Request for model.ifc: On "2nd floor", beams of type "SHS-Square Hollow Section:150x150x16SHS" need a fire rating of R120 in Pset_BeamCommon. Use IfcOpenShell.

First a look at what the model holds.

```python
import ifcopenshell
import ifcopenshell.util.element

model = ifcopenshell.open("model.ifc")
print(model.schema)
storey = next(s for s in model.by_type("IfcBuildingStorey") if s.Name == "2nd floor")
beams = [e for e in ifcopenshell.util.element.get_decomposition(storey) if e.is_a("IfcBeam")]
seen = {}
for e in beams:
    element_type = ifcopenshell.util.element.get_type(e)
    key = (element_type.Name if element_type != e and element_type else None, ifcopenshell.util.element.get_pset(e, "Pset_BeamCommon", "FireRating"))
    seen[key] = seen.get(key, 0) + 1
for (name, value), count in sorted(seen.items(), key=str):
    print(count, "x", name, "|", value)
```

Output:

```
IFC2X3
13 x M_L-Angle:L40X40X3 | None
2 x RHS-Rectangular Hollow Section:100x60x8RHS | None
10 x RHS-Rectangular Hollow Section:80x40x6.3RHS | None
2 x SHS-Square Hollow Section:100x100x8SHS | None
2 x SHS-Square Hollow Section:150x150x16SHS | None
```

```python
import ifcopenshell
import ifcopenshell.api.pset
import ifcopenshell.util.element

model = ifcopenshell.open("model.ifc")

storey = next(s for s in model.by_type("IfcBuildingStorey") if s.Name == "2nd floor")
beams = [e for e in ifcopenshell.util.element.get_decomposition(storey) if e.is_a("IfcBeam")]

count = 0
for e in beams:
    element_type = ifcopenshell.util.element.get_type(e)
    if element_type in (None, e) or element_type.Name != "SHS-Square Hollow Section:150x150x16SHS":
        continue
    # add_pset returns the element's existing set when there is one.
    pset = ifcopenshell.api.pset.add_pset(model, product=e, name="Pset_BeamCommon")
    ifcopenshell.api.pset.edit_pset(model, pset=pset, properties={"FireRating": "R120"})
    count += 1

print(count, "beams updated")

model.write("model_updated.ifc")
```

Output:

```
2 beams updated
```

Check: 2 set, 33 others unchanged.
